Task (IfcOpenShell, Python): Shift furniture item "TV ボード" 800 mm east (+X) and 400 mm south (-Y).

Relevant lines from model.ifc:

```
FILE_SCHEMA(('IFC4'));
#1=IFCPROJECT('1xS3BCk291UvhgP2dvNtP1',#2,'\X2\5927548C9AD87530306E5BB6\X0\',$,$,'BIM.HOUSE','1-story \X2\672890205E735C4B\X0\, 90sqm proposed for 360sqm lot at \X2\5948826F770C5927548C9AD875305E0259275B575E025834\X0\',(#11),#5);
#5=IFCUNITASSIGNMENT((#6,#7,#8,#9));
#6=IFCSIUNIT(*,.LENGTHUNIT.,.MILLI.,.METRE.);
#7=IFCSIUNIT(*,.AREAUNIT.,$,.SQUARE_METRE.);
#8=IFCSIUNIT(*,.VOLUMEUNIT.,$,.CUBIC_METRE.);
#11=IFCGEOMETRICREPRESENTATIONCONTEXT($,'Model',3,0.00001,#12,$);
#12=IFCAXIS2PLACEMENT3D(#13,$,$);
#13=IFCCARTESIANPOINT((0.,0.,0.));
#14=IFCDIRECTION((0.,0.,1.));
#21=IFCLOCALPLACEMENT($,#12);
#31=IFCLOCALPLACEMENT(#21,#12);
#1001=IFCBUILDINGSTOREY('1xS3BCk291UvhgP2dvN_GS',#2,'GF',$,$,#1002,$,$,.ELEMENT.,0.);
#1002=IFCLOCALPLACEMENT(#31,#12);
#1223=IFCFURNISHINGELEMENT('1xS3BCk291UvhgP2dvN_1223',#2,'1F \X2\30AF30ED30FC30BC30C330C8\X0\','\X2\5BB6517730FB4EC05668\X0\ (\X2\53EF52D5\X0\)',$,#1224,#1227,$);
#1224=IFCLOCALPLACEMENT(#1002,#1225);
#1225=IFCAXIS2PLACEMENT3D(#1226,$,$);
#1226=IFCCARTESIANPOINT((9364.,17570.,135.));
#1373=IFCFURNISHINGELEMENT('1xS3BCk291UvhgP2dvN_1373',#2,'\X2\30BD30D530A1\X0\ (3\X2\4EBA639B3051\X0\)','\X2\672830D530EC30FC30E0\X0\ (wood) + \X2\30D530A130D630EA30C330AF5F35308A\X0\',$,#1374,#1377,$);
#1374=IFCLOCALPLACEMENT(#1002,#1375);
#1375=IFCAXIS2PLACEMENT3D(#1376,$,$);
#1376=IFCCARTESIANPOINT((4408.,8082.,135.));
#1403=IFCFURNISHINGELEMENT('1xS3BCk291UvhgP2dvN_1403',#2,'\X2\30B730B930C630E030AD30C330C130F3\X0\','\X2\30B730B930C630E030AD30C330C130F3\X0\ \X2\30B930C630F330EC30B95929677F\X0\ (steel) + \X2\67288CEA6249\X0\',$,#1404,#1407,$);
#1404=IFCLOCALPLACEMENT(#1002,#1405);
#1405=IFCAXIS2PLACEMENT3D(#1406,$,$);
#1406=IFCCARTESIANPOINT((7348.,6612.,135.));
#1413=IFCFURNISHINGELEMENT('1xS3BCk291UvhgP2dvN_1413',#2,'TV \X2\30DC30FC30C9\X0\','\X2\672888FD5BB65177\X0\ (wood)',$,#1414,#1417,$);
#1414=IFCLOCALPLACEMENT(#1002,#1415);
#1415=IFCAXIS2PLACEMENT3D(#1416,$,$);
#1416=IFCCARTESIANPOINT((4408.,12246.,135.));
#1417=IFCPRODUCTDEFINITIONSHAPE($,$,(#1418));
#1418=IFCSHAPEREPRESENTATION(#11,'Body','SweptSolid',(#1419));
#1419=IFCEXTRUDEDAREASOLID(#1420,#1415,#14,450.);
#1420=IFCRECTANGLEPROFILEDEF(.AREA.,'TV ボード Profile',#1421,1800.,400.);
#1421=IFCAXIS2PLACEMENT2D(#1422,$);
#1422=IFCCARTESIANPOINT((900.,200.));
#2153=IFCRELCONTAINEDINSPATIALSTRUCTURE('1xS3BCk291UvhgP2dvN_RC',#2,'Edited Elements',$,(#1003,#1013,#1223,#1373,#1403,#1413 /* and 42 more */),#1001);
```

```python
import ifcopenshell
import ifcopenshell.api.geometry
import ifcopenshell.util.placement

model = ifcopenshell.open("model.ifc")

item = model.by_id(1413)
matrix = ifcopenshell.util.placement.get_local_placement(item.ObjectPlacement)
matrix[0, 3] += 800.0
matrix[1, 3] -= 400.0
ifcopenshell.api.geometry.edit_object_placement(model, product=item, matrix=matrix, is_si=False)

print(ifcopenshell.util.placement.get_local_placement(item.ObjectPlacement).round(3) + 0.0)

model.write("model_rev.ifc")
```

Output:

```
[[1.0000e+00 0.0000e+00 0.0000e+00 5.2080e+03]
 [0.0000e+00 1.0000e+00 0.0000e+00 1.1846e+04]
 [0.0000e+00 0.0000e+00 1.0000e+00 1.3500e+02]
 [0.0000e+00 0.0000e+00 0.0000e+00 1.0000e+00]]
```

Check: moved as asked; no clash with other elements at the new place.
